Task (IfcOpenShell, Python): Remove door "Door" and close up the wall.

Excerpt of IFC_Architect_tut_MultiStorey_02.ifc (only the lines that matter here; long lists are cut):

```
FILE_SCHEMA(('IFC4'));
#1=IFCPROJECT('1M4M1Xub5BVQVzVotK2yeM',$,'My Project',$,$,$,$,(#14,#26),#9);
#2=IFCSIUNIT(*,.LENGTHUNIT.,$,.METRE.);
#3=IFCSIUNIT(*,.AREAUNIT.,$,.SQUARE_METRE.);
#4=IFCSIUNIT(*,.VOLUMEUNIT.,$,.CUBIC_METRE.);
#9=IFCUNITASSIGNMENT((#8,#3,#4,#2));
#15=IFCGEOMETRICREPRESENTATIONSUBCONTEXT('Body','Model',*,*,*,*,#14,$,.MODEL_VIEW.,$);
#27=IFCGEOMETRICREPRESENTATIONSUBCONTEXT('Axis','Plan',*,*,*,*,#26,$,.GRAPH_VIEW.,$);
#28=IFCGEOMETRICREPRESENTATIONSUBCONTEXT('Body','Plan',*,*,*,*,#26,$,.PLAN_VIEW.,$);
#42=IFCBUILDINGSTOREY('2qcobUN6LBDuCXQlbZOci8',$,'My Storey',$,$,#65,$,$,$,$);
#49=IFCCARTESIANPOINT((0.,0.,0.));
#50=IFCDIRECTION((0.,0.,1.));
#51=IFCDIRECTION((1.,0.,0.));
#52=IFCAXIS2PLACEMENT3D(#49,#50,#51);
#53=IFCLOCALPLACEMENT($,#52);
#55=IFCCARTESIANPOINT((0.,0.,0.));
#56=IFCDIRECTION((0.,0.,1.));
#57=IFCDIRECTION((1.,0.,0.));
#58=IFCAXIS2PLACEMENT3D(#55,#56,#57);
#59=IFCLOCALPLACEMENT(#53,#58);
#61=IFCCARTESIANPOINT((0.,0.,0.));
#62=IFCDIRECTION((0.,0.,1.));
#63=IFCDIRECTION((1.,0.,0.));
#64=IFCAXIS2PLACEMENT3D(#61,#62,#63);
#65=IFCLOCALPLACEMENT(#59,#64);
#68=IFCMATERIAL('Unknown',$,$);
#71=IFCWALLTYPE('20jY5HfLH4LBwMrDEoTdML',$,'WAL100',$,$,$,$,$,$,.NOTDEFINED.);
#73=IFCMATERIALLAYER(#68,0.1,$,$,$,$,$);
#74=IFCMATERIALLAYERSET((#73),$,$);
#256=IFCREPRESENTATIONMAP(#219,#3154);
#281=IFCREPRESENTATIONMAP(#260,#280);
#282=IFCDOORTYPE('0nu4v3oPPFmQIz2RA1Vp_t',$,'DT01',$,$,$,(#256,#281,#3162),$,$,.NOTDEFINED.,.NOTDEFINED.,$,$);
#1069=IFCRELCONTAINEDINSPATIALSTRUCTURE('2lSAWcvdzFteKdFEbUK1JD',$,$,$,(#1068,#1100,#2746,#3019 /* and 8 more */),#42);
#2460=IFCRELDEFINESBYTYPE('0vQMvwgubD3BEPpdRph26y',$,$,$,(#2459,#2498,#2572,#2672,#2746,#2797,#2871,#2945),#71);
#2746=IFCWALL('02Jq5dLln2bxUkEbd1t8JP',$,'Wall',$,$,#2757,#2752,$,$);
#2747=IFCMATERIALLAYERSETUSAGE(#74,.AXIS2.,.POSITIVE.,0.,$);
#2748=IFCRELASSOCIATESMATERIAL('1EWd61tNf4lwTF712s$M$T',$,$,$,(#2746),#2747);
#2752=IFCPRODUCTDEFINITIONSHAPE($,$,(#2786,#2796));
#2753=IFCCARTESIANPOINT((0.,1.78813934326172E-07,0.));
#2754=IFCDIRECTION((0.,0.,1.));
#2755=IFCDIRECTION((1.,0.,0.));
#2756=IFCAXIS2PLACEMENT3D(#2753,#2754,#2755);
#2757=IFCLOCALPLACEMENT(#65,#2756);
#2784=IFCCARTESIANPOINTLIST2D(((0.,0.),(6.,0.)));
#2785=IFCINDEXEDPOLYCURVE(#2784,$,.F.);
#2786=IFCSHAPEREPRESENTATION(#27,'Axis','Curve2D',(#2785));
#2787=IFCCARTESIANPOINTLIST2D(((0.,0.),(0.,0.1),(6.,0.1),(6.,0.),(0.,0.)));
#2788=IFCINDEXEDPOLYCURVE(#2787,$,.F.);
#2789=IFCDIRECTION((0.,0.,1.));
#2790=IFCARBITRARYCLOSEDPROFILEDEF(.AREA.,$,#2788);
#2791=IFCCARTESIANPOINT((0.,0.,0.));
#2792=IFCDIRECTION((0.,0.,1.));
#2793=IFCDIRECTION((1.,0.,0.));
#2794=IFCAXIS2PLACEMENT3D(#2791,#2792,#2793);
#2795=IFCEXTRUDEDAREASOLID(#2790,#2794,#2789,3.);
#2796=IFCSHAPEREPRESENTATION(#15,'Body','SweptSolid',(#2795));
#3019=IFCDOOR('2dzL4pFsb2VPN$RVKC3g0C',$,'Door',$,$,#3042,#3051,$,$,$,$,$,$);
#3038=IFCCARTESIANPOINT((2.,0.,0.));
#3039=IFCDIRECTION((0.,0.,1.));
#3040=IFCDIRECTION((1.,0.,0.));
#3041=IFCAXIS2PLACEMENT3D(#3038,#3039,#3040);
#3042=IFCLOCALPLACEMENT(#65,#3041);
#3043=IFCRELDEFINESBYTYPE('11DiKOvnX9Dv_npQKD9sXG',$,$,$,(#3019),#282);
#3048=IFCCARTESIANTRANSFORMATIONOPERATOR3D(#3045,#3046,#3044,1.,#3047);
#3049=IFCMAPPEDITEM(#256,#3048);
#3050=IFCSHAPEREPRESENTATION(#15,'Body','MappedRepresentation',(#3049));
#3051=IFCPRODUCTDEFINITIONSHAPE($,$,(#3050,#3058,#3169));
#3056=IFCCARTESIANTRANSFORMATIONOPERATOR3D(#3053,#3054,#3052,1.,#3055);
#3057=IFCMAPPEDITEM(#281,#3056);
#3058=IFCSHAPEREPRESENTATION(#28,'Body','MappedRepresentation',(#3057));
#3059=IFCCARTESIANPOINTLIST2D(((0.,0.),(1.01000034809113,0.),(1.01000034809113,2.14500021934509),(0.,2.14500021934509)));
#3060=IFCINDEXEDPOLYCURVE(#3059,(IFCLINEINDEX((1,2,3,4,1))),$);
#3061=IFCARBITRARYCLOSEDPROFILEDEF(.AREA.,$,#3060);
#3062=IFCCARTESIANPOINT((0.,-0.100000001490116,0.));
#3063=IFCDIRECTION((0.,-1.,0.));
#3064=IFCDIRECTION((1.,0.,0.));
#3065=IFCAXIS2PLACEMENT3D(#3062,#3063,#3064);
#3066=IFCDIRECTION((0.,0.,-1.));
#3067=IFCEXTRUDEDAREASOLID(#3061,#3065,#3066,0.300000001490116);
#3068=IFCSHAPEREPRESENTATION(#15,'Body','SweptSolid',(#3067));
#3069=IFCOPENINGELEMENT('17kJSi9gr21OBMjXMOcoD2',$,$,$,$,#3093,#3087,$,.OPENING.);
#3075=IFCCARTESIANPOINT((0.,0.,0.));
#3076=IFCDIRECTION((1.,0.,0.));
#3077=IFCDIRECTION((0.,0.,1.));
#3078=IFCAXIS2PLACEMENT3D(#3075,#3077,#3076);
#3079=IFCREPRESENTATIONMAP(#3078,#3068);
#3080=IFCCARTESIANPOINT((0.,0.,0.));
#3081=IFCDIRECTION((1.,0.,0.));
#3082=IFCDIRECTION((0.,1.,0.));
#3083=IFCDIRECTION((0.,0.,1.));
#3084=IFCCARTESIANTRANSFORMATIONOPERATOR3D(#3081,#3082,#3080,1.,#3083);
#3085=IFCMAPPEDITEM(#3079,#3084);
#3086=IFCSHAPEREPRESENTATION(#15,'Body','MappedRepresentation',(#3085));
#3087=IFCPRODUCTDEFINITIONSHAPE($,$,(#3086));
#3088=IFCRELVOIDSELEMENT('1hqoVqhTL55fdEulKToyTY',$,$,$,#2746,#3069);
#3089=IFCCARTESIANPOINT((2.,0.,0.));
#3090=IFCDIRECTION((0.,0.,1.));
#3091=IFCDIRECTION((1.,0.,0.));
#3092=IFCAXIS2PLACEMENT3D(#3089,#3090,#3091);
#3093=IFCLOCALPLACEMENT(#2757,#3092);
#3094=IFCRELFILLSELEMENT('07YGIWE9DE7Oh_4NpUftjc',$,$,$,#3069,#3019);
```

```python
import ifcopenshell
import ifcopenshell.api.feature
import ifcopenshell.api.root
import ifcopenshell.geom
import ifcopenshell.util.shape

model = ifcopenshell.open("IFC_Architect_tut_MultiStorey_02.ifc")
settings = ifcopenshell.geom.settings()


def volume(element):
    """Net volume in cubic metres, openings subtracted."""
    shape = ifcopenshell.geom.create_shape(settings, element)
    return ifcopenshell.util.shape.get_volume(shape.geometry)


door = model.by_id(3019)
opening = door.FillsVoids[0].RelatingOpeningElement
wall = opening.VoidsElements[0].RelatingBuildingElement
before = volume(wall)

ifcopenshell.api.root.remove_product(model, product=door)
ifcopenshell.api.feature.remove_feature(model, feature=opening)

after = volume(wall)

print(f"wall volume {before:.3f} -> {after:.3f} m3")

model.write("IFC_Architect_tut_MultiStorey_02_updated.ifc")
```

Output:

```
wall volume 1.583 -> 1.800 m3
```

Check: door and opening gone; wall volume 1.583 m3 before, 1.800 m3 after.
